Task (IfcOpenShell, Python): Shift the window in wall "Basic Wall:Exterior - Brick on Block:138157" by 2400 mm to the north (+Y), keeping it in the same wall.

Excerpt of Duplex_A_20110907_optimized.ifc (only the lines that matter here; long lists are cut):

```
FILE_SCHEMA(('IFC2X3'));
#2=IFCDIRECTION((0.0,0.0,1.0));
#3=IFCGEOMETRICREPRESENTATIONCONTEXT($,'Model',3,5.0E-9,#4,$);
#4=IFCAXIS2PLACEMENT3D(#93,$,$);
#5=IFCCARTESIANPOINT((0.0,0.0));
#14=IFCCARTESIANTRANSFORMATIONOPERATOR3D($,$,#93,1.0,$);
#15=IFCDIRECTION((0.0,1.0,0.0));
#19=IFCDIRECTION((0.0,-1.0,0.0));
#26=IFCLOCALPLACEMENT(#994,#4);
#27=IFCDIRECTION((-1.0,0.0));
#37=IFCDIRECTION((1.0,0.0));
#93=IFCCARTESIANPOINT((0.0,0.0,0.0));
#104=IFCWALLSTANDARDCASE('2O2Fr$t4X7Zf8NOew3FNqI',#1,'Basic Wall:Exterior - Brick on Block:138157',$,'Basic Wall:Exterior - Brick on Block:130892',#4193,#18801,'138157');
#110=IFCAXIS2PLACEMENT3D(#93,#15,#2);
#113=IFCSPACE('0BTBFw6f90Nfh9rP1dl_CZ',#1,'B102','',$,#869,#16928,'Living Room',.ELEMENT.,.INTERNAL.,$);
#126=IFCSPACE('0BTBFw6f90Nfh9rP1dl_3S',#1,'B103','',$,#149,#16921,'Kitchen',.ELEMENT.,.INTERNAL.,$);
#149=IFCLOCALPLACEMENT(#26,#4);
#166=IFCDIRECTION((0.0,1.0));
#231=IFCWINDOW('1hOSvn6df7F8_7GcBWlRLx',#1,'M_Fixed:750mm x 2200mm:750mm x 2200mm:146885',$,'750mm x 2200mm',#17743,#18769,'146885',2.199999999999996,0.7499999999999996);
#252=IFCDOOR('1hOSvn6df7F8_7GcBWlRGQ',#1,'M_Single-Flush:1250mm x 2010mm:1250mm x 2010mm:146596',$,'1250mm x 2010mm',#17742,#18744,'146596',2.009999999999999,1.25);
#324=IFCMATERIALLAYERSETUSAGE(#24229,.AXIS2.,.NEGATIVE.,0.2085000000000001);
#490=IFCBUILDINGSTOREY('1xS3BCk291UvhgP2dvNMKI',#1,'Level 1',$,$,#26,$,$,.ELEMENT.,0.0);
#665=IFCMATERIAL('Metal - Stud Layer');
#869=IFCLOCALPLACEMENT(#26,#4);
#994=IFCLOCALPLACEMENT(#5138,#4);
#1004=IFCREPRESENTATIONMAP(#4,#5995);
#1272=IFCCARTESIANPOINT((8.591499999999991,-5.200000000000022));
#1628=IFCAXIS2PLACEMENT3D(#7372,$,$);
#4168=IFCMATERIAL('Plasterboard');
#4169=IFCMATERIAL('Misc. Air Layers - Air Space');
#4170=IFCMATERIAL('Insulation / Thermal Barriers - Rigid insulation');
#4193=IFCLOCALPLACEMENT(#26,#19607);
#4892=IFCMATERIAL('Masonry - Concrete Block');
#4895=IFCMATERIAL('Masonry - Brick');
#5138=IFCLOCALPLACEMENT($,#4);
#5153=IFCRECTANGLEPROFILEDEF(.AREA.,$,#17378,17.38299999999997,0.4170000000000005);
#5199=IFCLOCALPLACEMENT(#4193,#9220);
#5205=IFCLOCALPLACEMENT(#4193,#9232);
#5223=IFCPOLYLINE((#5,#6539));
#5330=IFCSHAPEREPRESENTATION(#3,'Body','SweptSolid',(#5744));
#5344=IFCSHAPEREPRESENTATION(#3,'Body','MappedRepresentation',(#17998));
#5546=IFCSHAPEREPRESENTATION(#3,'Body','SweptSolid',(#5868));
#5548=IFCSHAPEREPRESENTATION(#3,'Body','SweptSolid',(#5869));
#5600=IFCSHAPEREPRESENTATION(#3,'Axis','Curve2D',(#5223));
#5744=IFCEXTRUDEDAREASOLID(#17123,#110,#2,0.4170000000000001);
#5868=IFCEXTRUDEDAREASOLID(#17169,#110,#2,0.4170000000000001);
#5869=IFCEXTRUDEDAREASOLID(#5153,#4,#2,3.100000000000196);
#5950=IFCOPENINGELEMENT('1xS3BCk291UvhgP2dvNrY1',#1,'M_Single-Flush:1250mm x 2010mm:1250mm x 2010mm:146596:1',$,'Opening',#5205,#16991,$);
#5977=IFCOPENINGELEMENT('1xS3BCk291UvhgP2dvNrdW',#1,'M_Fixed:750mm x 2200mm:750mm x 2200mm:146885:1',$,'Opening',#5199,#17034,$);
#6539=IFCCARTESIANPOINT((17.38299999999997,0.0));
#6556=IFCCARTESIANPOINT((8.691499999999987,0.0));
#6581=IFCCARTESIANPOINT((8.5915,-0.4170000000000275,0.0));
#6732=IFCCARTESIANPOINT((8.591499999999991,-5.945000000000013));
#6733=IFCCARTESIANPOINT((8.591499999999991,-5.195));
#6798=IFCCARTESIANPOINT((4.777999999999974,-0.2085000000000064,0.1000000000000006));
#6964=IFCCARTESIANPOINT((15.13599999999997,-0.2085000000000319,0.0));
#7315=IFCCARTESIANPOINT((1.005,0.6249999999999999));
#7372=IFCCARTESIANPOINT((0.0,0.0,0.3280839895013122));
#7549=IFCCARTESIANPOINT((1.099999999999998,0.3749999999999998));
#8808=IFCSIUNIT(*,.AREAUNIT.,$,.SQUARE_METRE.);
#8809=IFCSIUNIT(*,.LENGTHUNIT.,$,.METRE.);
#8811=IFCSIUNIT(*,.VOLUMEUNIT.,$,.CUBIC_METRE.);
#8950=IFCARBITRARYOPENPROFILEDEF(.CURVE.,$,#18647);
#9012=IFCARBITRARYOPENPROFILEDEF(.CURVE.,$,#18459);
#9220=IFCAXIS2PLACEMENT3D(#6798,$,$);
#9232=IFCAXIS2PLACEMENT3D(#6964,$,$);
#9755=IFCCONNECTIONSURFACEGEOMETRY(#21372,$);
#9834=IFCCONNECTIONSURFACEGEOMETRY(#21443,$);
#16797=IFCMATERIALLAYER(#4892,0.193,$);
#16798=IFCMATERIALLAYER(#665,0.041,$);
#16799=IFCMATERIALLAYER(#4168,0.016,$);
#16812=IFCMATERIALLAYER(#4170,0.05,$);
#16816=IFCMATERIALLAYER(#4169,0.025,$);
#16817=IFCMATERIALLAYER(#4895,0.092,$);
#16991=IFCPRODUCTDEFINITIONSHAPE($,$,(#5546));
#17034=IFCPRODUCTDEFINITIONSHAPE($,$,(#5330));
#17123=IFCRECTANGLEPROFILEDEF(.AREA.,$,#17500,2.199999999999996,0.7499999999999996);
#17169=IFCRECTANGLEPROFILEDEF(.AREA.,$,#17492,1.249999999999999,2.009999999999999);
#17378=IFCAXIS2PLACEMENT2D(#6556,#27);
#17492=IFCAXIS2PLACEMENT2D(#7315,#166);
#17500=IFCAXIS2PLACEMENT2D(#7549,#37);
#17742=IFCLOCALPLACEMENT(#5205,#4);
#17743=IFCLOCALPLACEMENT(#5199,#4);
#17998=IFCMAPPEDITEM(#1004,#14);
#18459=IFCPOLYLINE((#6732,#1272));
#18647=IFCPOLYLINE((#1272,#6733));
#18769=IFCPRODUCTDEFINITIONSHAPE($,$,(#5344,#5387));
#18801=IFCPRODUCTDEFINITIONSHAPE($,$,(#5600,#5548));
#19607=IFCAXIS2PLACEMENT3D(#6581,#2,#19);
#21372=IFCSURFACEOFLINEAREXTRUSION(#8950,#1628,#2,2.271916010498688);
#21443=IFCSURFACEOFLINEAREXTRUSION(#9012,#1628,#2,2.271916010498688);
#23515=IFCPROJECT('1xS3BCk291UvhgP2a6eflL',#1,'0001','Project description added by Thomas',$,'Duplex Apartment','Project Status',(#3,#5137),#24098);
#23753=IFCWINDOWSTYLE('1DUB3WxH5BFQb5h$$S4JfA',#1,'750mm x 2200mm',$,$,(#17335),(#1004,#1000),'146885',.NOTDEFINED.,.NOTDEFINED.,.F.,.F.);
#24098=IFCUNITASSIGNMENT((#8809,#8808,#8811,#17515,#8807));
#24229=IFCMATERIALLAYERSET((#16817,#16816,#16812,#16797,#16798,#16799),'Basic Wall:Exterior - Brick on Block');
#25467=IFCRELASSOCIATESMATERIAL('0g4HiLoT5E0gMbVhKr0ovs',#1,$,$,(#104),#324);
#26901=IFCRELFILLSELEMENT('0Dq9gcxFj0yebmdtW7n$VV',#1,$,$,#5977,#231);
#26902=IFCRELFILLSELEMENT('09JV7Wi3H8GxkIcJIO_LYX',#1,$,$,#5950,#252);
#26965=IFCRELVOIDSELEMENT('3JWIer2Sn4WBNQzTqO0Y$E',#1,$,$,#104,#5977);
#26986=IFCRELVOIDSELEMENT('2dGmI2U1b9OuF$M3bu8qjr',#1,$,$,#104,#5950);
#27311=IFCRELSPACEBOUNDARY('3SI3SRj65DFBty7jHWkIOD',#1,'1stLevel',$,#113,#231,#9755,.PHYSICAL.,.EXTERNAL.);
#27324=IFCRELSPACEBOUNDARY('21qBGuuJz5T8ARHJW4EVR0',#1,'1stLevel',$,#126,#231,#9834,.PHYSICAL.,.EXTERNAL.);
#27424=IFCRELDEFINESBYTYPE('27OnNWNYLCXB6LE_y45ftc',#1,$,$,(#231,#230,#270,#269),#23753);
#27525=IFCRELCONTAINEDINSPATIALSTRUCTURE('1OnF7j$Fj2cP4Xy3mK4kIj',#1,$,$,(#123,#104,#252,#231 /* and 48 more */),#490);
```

```python
import numpy as np
import ifcopenshell
import ifcopenshell.api.geometry
import ifcopenshell.util.placement
import ifcopenshell.util.unit

model = ifcopenshell.open("Duplex_A_20110907_optimized.ifc")
unit_scale = ifcopenshell.util.unit.calculate_unit_scale(model)

window = model.by_guid("1hOSvn6df7F8_7GcBWlRLx")
opening = window.FillsVoids[0].RelatingOpeningElement
wall = opening.VoidsElements[0].RelatingBuildingElement

wall_matrix = ifcopenshell.util.placement.get_local_placement(wall.ObjectPlacement)
shift = wall_matrix[:3, 0] * -2.4 / unit_scale
before = ifcopenshell.util.placement.get_local_placement(window.ObjectPlacement)[:3, 3].copy()

# The window is placed relative to its opening, so it follows when the opening moves.
matrix = ifcopenshell.util.placement.get_local_placement(opening.ObjectPlacement)
matrix[:3, 3] += shift
ifcopenshell.api.geometry.edit_object_placement(
    model, product=opening, matrix=matrix, is_si=False, should_transform_children=True
)

# Space boundary surfaces are stored in each space's coordinates; move them too.
for rel in window.ProvidesBoundaries:
    if not rel.ConnectionGeometry:
        continue
    surface = rel.ConnectionGeometry.SurfaceOnRelatingElement
    space_matrix = ifcopenshell.util.placement.get_local_placement(rel.RelatingSpace.ObjectPlacement)
    point = np.array(surface.Position.Location.Coordinates) + space_matrix[:3, :3].T @ shift
    surface.Position = model.createIfcAxis2Placement3D(
        model.createIfcCartesianPoint(point.tolist()), surface.Position.Axis, surface.Position.RefDirection
    )

after = ifcopenshell.util.placement.get_local_placement(window.ObjectPlacement)[:3, 3]
print("window moved by", (after - before).round(3) + 0.0)

model.write("Duplex_A_20110907_optimized_updated.ifc")
```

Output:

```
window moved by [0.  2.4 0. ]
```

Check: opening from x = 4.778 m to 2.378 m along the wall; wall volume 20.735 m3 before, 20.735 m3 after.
